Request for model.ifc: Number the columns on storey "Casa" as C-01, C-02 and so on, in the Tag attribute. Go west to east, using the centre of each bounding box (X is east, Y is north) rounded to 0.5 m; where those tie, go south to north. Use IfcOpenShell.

First a look at what the model holds.

```python
import ifcopenshell
import ifcopenshell.util.element
import ifcopenshell.util.placement

model = ifcopenshell.open("model.ifc")
print(model.schema)
storey = next(s for s in model.by_type("IfcBuildingStorey") if s.Name == "Casa")
columns = [e for e in ifcopenshell.util.element.get_decomposition(storey) if e.is_a("IfcColumn")]
for e in sorted(columns, key=lambda e: e.id()):
    origin = ifcopenshell.util.placement.get_local_placement(e.ObjectPlacement)[:3, 3]
    print(e.id(), e.Tag, e.Name, origin.round(2) + 0.0, sep=" | ")
```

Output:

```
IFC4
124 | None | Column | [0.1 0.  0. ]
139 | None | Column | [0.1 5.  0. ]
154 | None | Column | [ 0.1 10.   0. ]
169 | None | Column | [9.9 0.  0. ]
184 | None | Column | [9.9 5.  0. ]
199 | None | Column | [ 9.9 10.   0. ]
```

```python
import ifcopenshell
import ifcopenshell.geom
import ifcopenshell.util.element
import ifcopenshell.util.shape

model = ifcopenshell.open("model.ifc")
settings = ifcopenshell.geom.settings()
settings.set("use-world-coords", True)


def centre(element):
    shape = ifcopenshell.geom.create_shape(settings, element)
    return ifcopenshell.util.shape.get_bbox_centroid(shape.geometry)


storey = next(s for s in model.by_type("IfcBuildingStorey") if s.Name == "Casa")
columns = [e for e in ifcopenshell.util.element.get_decomposition(storey) if e.is_a("IfcColumn")]

# Insertion points can sit at a corner or the storey origin, so sort by the geometry (in metres).
centres = {e: centre(e) for e in columns}
columns.sort(key=lambda e: (round(centres[e][0] / 0.5), centres[e][1]))

for i, e in enumerate(columns, start=1):
    number = f"C-{i:02d}"
    e.Tag = number
    print(e.id(), number)

model.write("model-out.ifc")
```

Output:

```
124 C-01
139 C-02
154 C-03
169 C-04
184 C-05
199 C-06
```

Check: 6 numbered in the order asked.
